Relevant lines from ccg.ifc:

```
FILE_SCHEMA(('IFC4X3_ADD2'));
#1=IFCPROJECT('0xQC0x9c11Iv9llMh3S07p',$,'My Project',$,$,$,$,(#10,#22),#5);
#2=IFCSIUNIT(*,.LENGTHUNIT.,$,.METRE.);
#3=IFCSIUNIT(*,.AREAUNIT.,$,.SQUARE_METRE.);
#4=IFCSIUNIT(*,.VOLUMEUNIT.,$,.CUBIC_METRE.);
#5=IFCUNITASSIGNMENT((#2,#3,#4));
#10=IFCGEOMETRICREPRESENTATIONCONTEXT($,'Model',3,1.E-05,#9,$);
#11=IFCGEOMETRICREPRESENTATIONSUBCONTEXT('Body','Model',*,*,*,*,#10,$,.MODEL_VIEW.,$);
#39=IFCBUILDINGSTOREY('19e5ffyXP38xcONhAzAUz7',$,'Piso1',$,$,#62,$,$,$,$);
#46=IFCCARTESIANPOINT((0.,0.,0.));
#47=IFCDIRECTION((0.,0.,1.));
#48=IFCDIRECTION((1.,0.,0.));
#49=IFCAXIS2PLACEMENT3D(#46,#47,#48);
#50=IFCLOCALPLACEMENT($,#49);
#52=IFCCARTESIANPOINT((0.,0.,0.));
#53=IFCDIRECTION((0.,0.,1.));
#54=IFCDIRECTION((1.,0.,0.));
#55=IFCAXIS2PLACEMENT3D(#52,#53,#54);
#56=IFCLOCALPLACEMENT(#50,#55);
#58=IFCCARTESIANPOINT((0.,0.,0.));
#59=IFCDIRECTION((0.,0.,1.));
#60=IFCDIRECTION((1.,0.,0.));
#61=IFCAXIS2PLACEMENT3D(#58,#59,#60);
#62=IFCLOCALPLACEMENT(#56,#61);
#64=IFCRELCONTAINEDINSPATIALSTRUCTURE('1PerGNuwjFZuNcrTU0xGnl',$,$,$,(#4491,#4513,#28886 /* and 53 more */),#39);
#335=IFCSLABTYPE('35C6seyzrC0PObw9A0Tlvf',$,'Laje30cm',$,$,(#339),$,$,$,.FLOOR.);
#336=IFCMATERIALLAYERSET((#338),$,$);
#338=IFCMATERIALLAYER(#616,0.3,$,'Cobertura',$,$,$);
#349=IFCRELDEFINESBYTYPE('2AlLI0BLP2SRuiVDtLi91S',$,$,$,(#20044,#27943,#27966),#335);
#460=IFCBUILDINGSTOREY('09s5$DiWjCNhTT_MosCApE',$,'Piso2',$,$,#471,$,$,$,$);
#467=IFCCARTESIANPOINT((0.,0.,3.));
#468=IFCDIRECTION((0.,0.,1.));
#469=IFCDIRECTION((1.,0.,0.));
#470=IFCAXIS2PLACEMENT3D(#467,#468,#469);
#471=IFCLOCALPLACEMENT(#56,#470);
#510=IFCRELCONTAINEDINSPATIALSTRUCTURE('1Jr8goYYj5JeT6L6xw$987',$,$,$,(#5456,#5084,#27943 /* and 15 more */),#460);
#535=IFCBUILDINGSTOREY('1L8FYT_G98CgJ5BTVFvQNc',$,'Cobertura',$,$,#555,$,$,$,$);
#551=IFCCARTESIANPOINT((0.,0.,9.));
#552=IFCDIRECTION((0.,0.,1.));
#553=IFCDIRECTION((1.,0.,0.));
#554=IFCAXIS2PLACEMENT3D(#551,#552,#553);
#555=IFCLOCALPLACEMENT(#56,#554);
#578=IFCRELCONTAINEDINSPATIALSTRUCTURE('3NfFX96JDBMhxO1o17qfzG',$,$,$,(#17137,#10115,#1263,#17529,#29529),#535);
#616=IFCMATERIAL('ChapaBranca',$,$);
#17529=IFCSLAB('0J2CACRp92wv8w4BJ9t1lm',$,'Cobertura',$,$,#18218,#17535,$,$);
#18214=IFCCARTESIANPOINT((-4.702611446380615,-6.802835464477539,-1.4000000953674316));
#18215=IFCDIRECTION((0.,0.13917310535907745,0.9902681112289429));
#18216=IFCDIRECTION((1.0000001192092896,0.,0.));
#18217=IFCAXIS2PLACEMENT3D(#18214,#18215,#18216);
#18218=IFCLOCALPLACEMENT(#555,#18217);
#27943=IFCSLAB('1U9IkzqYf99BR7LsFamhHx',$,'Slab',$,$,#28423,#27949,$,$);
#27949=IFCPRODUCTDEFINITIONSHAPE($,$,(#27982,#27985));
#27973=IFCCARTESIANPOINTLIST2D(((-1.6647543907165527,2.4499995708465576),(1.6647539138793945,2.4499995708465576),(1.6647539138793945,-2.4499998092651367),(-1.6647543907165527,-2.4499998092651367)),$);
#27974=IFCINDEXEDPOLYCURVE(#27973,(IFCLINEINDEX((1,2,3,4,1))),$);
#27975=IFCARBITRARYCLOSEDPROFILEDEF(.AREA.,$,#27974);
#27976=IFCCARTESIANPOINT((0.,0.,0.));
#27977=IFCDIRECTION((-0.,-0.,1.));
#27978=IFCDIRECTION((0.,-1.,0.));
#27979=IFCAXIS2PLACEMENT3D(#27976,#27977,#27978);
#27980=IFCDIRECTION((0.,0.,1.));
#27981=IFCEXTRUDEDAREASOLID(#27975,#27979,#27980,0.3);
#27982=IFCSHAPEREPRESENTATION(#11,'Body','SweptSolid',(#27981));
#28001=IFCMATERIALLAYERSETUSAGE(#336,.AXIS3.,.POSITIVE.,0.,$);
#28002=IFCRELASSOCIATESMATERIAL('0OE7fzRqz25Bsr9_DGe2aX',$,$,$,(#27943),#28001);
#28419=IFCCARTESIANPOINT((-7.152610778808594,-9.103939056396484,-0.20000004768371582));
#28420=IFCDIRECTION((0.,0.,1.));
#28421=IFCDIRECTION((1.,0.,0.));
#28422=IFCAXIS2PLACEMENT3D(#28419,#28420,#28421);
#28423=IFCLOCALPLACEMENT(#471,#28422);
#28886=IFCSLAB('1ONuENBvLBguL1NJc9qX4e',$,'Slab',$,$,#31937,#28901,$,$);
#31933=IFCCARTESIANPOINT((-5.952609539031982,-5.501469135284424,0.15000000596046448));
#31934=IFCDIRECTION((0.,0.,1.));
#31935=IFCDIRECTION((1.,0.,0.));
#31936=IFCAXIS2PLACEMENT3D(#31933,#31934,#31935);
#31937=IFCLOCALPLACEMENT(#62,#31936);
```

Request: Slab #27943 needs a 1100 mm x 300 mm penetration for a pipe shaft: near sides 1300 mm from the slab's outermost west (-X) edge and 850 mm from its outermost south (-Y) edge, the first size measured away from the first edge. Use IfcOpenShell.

```python
import numpy as np
import ifcopenshell
import ifcopenshell.api.feature
import ifcopenshell.api.geometry
import ifcopenshell.api.root
import ifcopenshell.geom
import ifcopenshell.util.placement
import ifcopenshell.util.representation
import ifcopenshell.util.shape
import ifcopenshell.util.unit

model = ifcopenshell.open("ccg.ifc")
unit_scale = ifcopenshell.util.unit.calculate_unit_scale(model)
settings = ifcopenshell.geom.settings()


def volume(element):
    """Net volume in cubic metres, openings subtracted."""
    shape = ifcopenshell.geom.create_shape(settings, element)
    return ifcopenshell.util.shape.get_volume(shape.geometry)


slab = model.by_guid("1U9IkzqYf99BR7LsFamhHx")
before = volume(slab)

# Extent in the slab's own axes, in metres. The edges named are its -X and -Y sides.
slab_shape = ifcopenshell.geom.create_shape(settings, slab)
vertices = ifcopenshell.util.shape.get_vertices(slab_shape.geometry)
x_min, y_min, bottom = vertices.min(axis=0)
top = vertices[:, 2].max()

opening = ifcopenshell.api.root.create_entity(model, ifc_class="IfcOpeningElement", name="Pipe shaft opening", predefined_type="OPENING")
context = ifcopenshell.util.representation.get_context(model, "Model", "Body", "MODEL_VIEW")
width, depth = 1.1, 0.3
outline = [(0.0, 0.0), (width, 0.0), (width, depth), (0.0, depth), (0.0, 0.0)]
# Overshoot both faces by 50 mm so the cut is clean.
shape = ifcopenshell.api.geometry.add_slab_representation(
    model, context=context, depth=top - bottom + 0.1, polyline=outline
)
ifcopenshell.api.geometry.assign_representation(model, product=opening, representation=shape)

matrix = ifcopenshell.util.placement.get_local_placement(slab.ObjectPlacement)
matrix[:, 3] = matrix @ np.append(np.array([x_min + 1.3, y_min + 0.85, bottom - 0.05]) / unit_scale, 1.0)
ifcopenshell.api.geometry.edit_object_placement(model, product=opening, matrix=matrix, is_si=False)
ifcopenshell.api.feature.add_feature(model, feature=opening, element=slab)

after = volume(slab)

print(f"slab volume {before:.3f} -> {after:.3f} m3")

model.write("ccg_rev.ifc")
```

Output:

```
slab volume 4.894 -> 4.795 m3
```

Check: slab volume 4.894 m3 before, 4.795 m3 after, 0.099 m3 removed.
